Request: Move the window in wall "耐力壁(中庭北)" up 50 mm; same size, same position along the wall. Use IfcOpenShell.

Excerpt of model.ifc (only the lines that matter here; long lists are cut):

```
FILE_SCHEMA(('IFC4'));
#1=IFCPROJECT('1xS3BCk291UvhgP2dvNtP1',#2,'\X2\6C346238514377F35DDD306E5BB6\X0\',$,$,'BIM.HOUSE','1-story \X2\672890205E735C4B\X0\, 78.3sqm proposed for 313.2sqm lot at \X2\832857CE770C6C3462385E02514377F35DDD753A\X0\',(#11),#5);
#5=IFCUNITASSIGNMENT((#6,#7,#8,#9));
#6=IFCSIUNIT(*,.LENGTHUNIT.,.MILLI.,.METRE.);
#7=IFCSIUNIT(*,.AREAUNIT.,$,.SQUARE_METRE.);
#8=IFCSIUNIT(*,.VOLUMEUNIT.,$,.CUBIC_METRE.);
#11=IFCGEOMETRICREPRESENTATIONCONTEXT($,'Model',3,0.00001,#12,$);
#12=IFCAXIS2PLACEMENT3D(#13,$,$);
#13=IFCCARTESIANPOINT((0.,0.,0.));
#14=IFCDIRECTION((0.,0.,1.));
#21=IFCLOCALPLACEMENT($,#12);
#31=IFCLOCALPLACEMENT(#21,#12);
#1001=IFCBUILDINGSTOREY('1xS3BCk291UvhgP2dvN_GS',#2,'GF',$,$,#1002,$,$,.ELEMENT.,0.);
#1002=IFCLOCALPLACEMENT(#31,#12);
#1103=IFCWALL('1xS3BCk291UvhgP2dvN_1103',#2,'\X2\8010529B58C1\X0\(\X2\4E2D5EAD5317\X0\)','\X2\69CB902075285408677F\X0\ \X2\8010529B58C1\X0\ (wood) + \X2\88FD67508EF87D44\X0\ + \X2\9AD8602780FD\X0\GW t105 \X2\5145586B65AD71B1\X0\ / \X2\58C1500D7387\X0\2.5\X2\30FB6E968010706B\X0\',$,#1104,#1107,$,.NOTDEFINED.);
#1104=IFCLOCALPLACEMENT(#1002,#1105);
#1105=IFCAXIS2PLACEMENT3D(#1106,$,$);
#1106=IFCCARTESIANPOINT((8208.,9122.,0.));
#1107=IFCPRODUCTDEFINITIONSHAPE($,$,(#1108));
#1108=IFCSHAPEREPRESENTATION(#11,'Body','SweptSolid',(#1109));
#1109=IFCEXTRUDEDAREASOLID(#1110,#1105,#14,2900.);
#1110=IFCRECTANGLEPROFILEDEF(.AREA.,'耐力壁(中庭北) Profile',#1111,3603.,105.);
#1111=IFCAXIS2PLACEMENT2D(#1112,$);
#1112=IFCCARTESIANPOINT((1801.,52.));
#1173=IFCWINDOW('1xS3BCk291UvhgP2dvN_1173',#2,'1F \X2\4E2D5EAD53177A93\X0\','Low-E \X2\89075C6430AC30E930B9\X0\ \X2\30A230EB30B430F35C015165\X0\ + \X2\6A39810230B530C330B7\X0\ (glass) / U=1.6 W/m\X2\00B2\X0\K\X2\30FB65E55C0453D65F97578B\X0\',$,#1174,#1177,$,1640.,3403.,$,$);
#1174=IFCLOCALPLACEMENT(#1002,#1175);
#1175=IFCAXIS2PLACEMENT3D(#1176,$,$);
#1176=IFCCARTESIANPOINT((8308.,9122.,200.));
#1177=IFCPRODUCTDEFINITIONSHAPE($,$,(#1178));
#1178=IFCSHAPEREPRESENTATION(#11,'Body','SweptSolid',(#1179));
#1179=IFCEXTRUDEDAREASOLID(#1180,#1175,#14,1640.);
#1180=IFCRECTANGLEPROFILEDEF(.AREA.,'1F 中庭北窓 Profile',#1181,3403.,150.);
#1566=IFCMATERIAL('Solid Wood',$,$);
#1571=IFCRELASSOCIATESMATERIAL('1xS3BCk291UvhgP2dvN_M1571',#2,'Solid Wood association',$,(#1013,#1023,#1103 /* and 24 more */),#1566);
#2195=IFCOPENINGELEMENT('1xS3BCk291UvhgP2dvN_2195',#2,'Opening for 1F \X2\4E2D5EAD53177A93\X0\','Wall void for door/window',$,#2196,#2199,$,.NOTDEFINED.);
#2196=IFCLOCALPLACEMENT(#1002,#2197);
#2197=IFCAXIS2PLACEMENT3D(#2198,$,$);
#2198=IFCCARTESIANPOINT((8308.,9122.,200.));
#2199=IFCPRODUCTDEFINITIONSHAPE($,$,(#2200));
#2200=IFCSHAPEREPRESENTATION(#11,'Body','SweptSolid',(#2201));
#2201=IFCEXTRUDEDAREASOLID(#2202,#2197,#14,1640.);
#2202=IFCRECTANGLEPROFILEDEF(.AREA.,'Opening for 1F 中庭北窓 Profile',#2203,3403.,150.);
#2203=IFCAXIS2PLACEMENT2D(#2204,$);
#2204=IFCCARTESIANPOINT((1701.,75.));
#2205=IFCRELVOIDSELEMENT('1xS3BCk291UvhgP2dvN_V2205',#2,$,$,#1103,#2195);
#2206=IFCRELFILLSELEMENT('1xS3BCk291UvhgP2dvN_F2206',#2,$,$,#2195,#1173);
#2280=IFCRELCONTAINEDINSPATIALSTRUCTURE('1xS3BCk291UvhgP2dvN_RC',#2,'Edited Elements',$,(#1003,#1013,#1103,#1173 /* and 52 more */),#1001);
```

```python
import numpy as np
import ifcopenshell
import ifcopenshell.api.geometry
import ifcopenshell.util.placement
import ifcopenshell.util.unit

model = ifcopenshell.open("model.ifc")
unit_scale = ifcopenshell.util.unit.calculate_unit_scale(model)

window = model.by_guid("1xS3BCk291UvhgP2dvN_1173")
opening = window.FillsVoids[0].RelatingOpeningElement
dz = 0.05 / unit_scale

shift = np.array([0.0, 0.0, dz])
# The window is not placed relative to its opening, so move both.
for product in (opening, window):
    matrix = ifcopenshell.util.placement.get_local_placement(product.ObjectPlacement)
    matrix[:3, 3] += shift
    ifcopenshell.api.geometry.edit_object_placement(model, product=product, matrix=matrix, is_si=False)

print(f"moved by {dz * unit_scale:+.3f} m")

model.write("model_rev.ifc")
```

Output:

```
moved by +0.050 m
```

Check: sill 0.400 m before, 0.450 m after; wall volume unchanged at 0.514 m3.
